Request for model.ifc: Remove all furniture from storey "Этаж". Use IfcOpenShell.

First a look at what the model holds.

```python
import ifcopenshell
import ifcopenshell.util.element

model = ifcopenshell.open("model.ifc")
print(model.schema)
storey = next(s for s in model.by_type("IfcBuildingStorey") if s.Name == "Этаж")
furniture = [e for e in ifcopenshell.util.element.get_decomposition(storey) if e.is_a("IfcFurnishingElement")]
seen = {}
for e in furniture:
    element_type = ifcopenshell.util.element.get_type(e)
    name = element_type.Name if element_type not in (None, e) else None
    seen[name] = seen.get(name, 0) + 1
for name, count in sorted(seen.items(), key=str):
    print(count, "x", name)
```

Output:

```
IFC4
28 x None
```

```python
import ifcopenshell
import ifcopenshell.api.root
import ifcopenshell.util.element

model = ifcopenshell.open("model.ifc")

storey = next(s for s in model.by_type("IfcBuildingStorey") if s.Name == "Этаж")
furniture = [e for e in ifcopenshell.util.element.get_decomposition(storey) if e.is_a("IfcFurnishingElement")]

for e in furniture:
    ifcopenshell.api.root.remove_product(model, product=e)
print(len(furniture), "removed")

model.write("model-out.ifc")
```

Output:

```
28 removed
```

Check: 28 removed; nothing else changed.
